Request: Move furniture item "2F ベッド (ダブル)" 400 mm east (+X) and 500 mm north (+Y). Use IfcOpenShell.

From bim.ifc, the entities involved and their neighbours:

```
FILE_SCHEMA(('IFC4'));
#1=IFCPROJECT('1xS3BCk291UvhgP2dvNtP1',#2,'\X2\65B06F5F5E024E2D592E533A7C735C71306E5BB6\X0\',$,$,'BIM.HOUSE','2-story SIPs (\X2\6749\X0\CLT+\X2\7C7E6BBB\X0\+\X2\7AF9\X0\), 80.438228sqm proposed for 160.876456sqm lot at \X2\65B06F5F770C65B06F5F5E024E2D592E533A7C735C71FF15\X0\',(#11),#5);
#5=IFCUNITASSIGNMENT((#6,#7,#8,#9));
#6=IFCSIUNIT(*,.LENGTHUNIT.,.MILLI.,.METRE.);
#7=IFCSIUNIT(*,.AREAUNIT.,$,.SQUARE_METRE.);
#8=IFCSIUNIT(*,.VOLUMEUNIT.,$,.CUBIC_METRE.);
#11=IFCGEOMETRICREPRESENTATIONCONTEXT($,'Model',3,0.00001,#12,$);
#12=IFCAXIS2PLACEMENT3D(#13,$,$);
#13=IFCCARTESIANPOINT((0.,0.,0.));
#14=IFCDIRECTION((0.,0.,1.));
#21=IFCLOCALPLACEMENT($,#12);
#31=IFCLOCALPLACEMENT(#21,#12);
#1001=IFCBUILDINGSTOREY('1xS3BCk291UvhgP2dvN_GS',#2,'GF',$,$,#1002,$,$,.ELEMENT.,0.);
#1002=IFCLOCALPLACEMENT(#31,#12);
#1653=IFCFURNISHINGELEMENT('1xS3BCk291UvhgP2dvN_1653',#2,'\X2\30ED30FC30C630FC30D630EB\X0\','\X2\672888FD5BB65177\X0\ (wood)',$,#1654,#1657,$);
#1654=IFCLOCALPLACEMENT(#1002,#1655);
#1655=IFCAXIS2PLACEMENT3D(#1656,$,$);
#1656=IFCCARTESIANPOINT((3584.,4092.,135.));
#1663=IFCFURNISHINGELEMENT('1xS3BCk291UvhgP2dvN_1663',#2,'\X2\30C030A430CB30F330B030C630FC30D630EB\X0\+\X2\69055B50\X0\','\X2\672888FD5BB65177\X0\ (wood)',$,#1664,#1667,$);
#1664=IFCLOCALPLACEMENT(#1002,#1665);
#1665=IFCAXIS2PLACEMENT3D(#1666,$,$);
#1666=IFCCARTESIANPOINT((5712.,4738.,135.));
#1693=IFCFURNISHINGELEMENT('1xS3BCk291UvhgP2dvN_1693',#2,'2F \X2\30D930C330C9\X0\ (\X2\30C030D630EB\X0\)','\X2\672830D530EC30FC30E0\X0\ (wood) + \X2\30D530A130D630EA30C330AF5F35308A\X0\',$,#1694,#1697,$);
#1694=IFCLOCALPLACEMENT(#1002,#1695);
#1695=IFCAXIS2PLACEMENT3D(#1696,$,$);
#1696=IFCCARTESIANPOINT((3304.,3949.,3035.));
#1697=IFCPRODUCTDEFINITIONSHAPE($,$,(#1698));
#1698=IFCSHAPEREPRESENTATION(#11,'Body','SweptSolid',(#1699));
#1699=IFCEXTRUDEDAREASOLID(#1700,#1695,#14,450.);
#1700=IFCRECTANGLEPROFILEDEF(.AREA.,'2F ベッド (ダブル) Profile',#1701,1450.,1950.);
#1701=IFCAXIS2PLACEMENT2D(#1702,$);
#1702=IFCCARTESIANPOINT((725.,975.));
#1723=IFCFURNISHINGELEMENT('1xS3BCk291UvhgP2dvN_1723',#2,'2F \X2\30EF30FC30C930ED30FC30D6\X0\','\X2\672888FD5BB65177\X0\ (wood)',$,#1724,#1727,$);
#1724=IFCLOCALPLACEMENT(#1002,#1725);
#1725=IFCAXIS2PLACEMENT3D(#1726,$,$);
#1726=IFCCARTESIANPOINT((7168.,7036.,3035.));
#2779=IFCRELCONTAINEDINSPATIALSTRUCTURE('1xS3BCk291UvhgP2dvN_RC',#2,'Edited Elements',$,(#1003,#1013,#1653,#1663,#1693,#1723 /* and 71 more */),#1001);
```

```python
import ifcopenshell
import ifcopenshell.api.geometry
import ifcopenshell.util.placement

model = ifcopenshell.open("bim.ifc")

item = model.by_guid("1xS3BCk291UvhgP2dvN_1693")
matrix = ifcopenshell.util.placement.get_local_placement(item.ObjectPlacement)
matrix[0, 3] += 400.0
matrix[1, 3] += 500.0
ifcopenshell.api.geometry.edit_object_placement(model, product=item, matrix=matrix, is_si=False)

print(ifcopenshell.util.placement.get_local_placement(item.ObjectPlacement).round(3) + 0.0)

model.write("bim_updated.ifc")
```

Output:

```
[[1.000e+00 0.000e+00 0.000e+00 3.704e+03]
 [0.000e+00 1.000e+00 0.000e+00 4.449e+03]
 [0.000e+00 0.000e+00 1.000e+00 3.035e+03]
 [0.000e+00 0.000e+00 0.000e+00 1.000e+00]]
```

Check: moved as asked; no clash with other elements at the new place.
